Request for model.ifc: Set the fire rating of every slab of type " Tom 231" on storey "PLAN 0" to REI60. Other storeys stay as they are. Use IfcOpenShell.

First a look at what the model holds.

```python
import ifcopenshell
import ifcopenshell.util.element

model = ifcopenshell.open("model.ifc")
print(model.schema)
storey = next(s for s in model.by_type("IfcBuildingStorey") if s.Name == "PLAN 0")
slabs = [e for e in ifcopenshell.util.element.get_decomposition(storey) if e.is_a("IfcSlab")]
seen = {}
for e in slabs:
    element_type = ifcopenshell.util.element.get_type(e)
    key = (element_type.Name if element_type != e and element_type else None, ifcopenshell.util.element.get_pset(e, "Pset_SlabCommon", "FireRating"))
    seen[key] = seen.get(key, 0) + 1
for (name, value), count in sorted(seen.items(), key=str):
    print(count, "x", name, "|", value)
```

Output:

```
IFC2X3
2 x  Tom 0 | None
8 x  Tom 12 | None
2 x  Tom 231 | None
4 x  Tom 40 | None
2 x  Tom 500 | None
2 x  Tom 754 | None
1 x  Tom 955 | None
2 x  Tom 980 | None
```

```python
import ifcopenshell
import ifcopenshell.api.pset
import ifcopenshell.util.element

model = ifcopenshell.open("model.ifc")

storey = next(s for s in model.by_type("IfcBuildingStorey") if s.Name == "PLAN 0")
slabs = [e for e in ifcopenshell.util.element.get_decomposition(storey) if e.is_a("IfcSlab")]

count = 0
for e in slabs:
    element_type = ifcopenshell.util.element.get_type(e)
    if element_type in (None, e) or element_type.Name != " Tom 231":
        continue
    # add_pset returns the element's existing set when there is one.
    pset = ifcopenshell.api.pset.add_pset(model, product=e, name="Pset_SlabCommon")
    ifcopenshell.api.pset.edit_pset(model, pset=pset, properties={"FireRating": "REI60"})
    count += 1

print(count, "slabs updated")

model.write("model_updated.ifc")
```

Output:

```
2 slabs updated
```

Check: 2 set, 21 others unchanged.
